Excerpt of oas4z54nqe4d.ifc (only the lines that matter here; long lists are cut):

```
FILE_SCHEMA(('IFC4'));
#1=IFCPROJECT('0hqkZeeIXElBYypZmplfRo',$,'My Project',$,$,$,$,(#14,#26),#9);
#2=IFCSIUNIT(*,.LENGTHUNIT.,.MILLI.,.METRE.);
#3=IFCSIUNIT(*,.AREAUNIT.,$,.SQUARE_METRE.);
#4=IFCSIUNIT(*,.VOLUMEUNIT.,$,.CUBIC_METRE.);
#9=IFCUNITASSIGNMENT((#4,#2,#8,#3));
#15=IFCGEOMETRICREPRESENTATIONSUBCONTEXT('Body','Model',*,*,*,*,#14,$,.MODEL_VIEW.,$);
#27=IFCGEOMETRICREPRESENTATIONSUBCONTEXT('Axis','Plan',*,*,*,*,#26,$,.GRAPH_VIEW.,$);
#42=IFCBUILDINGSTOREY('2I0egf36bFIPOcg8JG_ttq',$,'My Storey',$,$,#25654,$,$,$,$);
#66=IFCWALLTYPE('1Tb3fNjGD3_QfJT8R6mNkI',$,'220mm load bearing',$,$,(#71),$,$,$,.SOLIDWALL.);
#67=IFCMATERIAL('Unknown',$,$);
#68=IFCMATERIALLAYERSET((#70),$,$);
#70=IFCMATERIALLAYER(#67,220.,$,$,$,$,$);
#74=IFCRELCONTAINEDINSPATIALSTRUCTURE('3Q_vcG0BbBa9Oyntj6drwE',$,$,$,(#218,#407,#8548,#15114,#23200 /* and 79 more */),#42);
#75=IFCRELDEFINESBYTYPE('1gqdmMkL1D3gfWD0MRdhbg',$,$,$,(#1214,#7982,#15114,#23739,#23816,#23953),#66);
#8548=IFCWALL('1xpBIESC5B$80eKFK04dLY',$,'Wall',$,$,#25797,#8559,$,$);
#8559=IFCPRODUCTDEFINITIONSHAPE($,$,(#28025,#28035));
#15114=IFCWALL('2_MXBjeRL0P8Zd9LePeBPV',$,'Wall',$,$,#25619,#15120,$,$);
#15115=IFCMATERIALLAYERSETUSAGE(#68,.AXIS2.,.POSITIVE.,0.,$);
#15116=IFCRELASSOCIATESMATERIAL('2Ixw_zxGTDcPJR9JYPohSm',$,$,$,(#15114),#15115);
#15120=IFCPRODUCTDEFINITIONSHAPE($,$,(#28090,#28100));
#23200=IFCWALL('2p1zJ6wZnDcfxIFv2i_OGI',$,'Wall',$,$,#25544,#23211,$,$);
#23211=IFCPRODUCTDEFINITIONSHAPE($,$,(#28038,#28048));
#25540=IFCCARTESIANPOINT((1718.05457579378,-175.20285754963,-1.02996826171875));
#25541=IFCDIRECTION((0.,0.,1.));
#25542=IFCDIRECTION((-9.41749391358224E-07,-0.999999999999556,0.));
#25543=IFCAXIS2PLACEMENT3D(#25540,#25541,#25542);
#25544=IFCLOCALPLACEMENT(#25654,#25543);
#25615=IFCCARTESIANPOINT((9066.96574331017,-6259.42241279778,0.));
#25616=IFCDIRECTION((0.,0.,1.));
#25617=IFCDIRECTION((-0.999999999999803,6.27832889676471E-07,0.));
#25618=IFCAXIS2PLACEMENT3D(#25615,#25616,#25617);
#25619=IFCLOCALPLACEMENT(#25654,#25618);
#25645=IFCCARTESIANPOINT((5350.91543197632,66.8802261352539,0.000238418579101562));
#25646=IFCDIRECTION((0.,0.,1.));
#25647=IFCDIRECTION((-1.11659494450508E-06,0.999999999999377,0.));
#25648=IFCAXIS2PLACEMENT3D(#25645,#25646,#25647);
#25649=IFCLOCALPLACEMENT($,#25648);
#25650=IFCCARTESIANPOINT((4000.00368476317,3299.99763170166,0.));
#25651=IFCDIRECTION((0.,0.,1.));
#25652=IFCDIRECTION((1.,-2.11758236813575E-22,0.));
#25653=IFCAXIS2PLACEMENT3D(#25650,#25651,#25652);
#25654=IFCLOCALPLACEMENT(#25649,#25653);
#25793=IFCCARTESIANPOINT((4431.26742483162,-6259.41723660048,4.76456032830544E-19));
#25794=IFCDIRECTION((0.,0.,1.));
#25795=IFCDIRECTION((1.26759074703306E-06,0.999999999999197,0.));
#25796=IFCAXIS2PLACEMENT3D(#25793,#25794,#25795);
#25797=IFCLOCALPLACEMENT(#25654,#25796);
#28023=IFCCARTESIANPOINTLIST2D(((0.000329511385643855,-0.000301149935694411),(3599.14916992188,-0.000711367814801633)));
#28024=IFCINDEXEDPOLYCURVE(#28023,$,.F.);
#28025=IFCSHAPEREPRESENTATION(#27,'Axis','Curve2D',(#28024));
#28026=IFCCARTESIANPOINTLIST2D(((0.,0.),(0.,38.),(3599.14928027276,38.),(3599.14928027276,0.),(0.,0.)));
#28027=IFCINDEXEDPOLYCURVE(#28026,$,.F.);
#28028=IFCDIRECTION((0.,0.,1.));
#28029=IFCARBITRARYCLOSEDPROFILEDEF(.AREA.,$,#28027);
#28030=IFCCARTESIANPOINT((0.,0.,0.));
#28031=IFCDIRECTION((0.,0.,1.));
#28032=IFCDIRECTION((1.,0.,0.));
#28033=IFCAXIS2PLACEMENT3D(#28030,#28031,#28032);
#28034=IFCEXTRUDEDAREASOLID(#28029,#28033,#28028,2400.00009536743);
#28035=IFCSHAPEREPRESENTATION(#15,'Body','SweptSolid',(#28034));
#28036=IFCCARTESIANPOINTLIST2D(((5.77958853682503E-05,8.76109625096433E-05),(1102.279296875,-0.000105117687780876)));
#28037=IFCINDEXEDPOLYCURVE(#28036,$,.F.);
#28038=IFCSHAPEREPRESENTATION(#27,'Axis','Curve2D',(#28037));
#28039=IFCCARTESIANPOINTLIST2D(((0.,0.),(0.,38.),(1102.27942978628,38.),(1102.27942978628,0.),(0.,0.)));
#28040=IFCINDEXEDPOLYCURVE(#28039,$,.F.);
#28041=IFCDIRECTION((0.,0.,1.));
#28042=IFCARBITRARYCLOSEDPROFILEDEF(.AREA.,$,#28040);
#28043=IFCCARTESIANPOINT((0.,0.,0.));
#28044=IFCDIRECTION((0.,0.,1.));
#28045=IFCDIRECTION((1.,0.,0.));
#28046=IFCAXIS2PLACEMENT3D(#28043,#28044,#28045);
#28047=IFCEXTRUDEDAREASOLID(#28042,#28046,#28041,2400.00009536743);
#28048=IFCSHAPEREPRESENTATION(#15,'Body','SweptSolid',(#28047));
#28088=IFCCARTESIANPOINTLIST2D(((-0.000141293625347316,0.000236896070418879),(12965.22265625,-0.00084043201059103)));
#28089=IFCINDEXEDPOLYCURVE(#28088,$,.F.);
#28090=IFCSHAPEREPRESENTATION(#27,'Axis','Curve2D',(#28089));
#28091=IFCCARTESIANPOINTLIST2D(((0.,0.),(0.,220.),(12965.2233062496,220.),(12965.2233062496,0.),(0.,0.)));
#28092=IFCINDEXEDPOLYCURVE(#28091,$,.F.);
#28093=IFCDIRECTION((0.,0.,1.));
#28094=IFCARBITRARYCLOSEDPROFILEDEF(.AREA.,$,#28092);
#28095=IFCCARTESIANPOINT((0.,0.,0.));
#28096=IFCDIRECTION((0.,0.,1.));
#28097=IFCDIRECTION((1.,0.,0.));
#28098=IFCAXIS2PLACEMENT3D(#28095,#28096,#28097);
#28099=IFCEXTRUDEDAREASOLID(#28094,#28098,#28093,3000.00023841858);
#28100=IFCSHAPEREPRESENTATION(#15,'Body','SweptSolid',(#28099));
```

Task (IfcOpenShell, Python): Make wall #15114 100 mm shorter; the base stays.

```python
import ifcopenshell
import ifcopenshell.geom
import ifcopenshell.util.representation
import ifcopenshell.util.shape
import ifcopenshell.util.unit

model = ifcopenshell.open("oas4z54nqe4d.ifc")
unit_scale = ifcopenshell.util.unit.calculate_unit_scale(model)
settings = ifcopenshell.geom.settings()


def volume(element):
    """Net volume in cubic metres, openings subtracted."""
    shape = ifcopenshell.geom.create_shape(settings, element)
    return ifcopenshell.util.shape.get_volume(shape.geometry)


wall = model.by_guid("2_MXBjeRL0P8Zd9LePeBPV")
before = volume(wall)

body = ifcopenshell.util.representation.get_representation(wall, "Model", "Body")
solid = body.Items[0]
old_height = solid.Depth
solid.Depth -= 0.1 / unit_scale
after = volume(wall)

print(f"height {old_height:g} -> {solid.Depth:g}, volume {before:.3f} -> {after:.3f} m3")

model.write("oas4z54nqe4d_rev.ifc")
```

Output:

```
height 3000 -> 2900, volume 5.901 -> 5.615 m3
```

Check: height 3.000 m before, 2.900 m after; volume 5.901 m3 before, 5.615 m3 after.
